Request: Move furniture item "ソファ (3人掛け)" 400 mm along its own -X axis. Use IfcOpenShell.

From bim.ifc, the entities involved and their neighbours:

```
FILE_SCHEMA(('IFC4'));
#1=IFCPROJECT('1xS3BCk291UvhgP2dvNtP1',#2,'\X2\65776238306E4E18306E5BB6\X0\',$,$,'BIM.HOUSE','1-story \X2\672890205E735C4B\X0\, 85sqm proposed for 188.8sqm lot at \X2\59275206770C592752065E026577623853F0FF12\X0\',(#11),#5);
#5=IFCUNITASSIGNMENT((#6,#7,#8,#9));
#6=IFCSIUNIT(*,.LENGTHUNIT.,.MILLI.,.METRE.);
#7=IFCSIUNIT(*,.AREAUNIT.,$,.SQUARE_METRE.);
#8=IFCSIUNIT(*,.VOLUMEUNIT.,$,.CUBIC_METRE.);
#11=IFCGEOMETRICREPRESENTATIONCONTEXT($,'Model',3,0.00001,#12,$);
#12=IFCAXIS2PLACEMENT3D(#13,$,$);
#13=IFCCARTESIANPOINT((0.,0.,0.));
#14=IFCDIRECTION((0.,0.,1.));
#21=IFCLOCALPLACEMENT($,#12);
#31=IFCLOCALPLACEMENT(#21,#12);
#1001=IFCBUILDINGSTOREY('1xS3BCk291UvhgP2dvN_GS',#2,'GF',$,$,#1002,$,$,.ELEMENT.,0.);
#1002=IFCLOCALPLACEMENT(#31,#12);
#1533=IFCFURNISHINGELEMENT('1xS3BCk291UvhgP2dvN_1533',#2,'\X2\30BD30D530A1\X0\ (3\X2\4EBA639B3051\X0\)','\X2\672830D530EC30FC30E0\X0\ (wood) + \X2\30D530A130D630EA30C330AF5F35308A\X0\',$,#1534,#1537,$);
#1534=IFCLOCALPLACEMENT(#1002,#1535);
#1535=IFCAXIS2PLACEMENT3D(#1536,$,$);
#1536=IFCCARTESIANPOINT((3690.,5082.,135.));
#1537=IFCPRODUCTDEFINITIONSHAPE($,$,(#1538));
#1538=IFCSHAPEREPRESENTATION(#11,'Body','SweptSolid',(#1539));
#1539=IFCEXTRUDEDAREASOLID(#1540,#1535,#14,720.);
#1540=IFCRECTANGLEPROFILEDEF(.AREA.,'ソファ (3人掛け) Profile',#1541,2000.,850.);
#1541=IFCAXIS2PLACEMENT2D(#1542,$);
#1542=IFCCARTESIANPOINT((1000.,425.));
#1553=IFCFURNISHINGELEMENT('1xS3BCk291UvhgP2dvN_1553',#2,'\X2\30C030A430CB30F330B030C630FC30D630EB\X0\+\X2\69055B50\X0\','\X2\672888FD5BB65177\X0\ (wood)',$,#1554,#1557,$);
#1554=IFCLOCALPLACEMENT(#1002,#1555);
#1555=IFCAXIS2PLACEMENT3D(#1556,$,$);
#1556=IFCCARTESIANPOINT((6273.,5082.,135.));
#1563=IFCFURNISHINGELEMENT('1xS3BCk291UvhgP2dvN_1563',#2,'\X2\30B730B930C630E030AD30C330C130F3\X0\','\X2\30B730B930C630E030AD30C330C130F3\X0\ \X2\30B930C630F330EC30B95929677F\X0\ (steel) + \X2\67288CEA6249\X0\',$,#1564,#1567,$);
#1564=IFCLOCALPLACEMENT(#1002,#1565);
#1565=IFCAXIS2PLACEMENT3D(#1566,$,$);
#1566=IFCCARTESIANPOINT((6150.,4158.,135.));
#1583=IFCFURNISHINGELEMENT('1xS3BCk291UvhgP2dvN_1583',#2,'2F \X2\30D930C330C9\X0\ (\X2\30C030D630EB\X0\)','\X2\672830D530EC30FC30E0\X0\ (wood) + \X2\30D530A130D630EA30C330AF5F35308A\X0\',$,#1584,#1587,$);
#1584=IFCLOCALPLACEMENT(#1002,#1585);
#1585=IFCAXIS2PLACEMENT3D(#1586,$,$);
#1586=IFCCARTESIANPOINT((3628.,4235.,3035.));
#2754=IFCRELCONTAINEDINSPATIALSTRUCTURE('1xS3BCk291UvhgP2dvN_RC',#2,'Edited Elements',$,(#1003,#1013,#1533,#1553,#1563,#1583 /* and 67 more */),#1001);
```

```python
import ifcopenshell
import ifcopenshell.api.geometry
import ifcopenshell.util.placement

model = ifcopenshell.open("bim.ifc")

item = model.by_guid("1xS3BCk291UvhgP2dvN_1533")
matrix = ifcopenshell.util.placement.get_local_placement(item.ObjectPlacement)
matrix[:3, 3] -= matrix[:3, 0] * 400.0
ifcopenshell.api.geometry.edit_object_placement(model, product=item, matrix=matrix, is_si=False)

print(ifcopenshell.util.placement.get_local_placement(item.ObjectPlacement).round(3) + 0.0)

model.write("bim_updated.ifc")
```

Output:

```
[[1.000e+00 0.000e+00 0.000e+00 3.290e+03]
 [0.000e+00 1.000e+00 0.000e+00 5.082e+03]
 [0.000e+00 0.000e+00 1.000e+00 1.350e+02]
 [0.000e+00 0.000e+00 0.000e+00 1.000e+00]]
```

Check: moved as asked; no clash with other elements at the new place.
